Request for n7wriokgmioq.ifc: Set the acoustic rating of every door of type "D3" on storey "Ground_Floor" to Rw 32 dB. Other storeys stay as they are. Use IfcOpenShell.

First a look at what the model holds.

```python
import ifcopenshell
import ifcopenshell.util.element

model = ifcopenshell.open("n7wriokgmioq.ifc")
print(model.schema)
storey = next(s for s in model.by_type("IfcBuildingStorey") if s.Name == "Ground_Floor")
doors = [e for e in ifcopenshell.util.element.get_decomposition(storey) if e.is_a("IfcDoor")]
seen = {}
for e in doors:
    element_type = ifcopenshell.util.element.get_type(e)
    key = (element_type.Name if element_type != e and element_type else None, ifcopenshell.util.element.get_pset(e, "Pset_DoorCommon", "AcousticRating"))
    seen[key] = seen.get(key, 0) + 1
for (name, value), count in sorted(seen.items(), key=str):
    print(count, "x", name, "|", value)
```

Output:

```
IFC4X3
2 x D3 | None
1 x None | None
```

```python
import ifcopenshell
import ifcopenshell.api.pset
import ifcopenshell.util.element

model = ifcopenshell.open("n7wriokgmioq.ifc")

storey = next(s for s in model.by_type("IfcBuildingStorey") if s.Name == "Ground_Floor")
doors = [e for e in ifcopenshell.util.element.get_decomposition(storey) if e.is_a("IfcDoor")]

count = 0
for e in doors:
    element_type = ifcopenshell.util.element.get_type(e)
    if element_type in (None, e) or element_type.Name != "D3":
        continue
    # add_pset returns the element's existing set when there is one.
    pset = ifcopenshell.api.pset.add_pset(model, product=e, name="Pset_DoorCommon")
    ifcopenshell.api.pset.edit_pset(model, pset=pset, properties={"AcousticRating": "Rw 32 dB"})
    count += 1

print(count, "doors updated")

model.write("n7wriokgmioq_edited.ifc")
```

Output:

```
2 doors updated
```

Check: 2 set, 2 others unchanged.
